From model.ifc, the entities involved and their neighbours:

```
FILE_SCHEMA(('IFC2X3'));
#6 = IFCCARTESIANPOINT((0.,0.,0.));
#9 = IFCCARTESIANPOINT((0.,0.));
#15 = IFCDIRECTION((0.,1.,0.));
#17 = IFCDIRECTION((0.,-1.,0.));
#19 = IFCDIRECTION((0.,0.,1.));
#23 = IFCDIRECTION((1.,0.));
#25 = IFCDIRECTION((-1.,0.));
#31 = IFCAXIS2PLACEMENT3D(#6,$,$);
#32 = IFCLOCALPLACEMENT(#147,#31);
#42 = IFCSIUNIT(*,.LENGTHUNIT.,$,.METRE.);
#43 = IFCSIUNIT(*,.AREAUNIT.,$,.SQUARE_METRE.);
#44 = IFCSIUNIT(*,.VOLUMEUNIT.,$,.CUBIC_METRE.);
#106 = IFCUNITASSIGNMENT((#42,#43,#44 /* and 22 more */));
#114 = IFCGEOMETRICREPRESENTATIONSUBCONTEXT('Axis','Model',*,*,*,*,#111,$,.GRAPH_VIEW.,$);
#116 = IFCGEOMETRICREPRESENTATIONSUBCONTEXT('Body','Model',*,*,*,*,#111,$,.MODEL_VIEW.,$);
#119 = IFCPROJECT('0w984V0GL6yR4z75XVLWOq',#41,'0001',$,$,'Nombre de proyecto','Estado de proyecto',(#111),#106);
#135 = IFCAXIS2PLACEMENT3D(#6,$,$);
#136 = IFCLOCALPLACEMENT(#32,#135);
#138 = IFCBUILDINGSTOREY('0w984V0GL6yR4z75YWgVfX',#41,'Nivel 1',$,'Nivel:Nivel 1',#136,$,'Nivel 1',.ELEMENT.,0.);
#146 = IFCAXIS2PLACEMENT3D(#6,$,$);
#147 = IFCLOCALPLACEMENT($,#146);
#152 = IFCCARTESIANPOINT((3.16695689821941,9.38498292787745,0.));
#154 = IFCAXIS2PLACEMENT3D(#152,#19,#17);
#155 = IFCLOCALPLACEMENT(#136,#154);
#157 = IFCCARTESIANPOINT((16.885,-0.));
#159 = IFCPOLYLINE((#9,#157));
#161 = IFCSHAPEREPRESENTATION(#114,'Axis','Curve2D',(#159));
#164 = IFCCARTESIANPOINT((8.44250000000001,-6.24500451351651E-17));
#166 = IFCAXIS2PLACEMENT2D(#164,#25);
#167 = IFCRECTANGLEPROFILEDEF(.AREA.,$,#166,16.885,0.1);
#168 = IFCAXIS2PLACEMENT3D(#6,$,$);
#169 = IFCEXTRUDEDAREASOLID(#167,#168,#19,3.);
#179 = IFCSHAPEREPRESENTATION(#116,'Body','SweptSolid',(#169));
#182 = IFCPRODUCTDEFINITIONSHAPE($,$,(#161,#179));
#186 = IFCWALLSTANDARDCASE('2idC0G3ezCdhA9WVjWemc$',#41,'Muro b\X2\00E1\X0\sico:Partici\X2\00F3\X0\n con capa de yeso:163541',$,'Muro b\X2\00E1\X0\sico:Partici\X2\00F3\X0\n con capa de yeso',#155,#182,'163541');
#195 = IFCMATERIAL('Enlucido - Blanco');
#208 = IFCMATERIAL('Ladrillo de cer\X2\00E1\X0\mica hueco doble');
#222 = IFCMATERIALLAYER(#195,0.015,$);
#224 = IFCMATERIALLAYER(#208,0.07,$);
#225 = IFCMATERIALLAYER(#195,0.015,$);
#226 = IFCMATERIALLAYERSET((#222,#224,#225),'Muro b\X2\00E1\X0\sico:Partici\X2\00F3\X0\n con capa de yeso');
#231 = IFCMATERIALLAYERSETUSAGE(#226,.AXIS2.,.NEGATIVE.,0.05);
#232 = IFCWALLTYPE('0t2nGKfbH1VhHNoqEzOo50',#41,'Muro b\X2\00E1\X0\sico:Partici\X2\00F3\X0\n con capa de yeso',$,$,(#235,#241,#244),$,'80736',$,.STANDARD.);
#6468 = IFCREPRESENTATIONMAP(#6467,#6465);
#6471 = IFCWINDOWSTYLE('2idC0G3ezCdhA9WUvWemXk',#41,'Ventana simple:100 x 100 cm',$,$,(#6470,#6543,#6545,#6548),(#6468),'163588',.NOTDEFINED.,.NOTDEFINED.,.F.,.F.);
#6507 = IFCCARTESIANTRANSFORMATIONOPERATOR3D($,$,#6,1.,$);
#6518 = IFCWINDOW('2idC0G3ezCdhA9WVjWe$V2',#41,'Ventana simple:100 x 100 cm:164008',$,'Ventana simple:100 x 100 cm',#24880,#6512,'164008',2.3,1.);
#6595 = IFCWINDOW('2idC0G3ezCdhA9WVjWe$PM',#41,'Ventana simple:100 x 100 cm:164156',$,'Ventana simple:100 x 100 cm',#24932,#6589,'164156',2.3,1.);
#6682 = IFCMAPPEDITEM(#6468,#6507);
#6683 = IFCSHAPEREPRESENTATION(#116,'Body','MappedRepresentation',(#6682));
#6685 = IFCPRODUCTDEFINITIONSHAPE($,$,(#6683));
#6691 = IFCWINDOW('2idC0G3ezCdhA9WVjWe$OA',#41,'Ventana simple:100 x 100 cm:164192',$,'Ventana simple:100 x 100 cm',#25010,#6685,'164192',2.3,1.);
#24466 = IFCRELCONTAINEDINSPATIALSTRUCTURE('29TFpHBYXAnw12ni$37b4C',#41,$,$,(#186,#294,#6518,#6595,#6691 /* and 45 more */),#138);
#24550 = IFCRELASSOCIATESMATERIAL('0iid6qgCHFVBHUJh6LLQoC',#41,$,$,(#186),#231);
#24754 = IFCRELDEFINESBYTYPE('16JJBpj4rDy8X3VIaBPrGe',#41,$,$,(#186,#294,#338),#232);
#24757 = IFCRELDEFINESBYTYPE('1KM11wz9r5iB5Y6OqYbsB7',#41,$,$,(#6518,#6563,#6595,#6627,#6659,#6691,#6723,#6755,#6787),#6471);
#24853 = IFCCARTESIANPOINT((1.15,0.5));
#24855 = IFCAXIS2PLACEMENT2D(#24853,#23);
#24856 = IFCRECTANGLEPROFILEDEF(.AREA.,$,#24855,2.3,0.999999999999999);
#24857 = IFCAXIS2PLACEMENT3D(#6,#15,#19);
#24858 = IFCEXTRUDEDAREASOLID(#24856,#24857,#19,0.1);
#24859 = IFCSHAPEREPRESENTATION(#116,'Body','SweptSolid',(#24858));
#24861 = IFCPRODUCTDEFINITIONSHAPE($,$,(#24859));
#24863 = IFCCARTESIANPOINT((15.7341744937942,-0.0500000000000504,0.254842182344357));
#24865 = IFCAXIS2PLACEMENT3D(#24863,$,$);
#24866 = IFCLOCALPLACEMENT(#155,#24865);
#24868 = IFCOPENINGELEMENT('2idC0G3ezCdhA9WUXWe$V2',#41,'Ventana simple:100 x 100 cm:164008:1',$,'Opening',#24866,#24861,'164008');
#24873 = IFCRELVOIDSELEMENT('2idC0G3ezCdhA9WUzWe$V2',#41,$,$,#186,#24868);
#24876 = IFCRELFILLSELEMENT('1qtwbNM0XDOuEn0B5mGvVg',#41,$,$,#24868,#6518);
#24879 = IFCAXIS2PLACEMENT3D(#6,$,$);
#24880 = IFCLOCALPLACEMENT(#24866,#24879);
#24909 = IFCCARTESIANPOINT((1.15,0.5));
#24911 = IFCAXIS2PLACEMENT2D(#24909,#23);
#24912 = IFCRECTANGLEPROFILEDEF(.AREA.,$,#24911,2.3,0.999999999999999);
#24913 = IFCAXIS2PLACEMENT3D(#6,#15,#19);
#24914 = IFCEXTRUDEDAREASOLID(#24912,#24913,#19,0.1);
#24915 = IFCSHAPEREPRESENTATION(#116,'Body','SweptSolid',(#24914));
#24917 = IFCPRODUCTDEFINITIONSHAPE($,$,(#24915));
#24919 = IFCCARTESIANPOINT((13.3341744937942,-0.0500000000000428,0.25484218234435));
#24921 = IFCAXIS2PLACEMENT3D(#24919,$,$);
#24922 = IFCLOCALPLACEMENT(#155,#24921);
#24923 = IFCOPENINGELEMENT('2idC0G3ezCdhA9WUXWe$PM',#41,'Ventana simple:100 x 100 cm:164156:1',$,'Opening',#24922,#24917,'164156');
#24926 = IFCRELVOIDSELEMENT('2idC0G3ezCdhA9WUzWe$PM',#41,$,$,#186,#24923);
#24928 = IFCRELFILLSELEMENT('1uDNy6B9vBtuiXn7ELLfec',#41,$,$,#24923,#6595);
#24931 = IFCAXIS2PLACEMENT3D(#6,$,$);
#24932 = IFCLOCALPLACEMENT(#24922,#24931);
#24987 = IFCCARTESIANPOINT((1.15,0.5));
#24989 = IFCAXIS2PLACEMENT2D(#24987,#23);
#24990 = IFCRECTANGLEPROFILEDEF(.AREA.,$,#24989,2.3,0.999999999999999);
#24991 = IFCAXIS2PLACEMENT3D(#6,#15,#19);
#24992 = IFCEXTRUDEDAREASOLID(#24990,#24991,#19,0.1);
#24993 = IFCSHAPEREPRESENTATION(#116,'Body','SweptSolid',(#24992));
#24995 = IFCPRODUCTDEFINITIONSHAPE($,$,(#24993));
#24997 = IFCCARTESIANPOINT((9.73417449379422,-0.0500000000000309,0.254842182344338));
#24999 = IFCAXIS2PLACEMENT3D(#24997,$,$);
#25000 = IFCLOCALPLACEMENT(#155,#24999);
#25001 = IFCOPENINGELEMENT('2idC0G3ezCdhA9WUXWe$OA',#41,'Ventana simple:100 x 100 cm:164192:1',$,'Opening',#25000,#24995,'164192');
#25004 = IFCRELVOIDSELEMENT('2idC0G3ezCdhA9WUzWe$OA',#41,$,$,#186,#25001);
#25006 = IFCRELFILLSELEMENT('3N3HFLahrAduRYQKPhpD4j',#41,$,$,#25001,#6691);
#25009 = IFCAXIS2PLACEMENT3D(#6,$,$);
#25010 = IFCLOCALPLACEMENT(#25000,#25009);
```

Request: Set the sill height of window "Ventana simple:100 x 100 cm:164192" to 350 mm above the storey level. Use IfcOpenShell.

```python
import numpy as np
import ifcopenshell
import ifcopenshell.api.geometry
import ifcopenshell.geom
import ifcopenshell.util.element
import ifcopenshell.util.placement
import ifcopenshell.util.shape
import ifcopenshell.util.unit

model = ifcopenshell.open("model.ifc")
unit_scale = ifcopenshell.util.unit.calculate_unit_scale(model)

window = model.by_guid("2idC0G3ezCdhA9WVjWe$OA")
opening = window.FillsVoids[0].RelatingOpeningElement
storey = ifcopenshell.util.element.get_container(window, ifc_class="IfcBuildingStorey")
level = ifcopenshell.util.placement.get_local_placement(storey.ObjectPlacement)[2, 3]

# The opening's origin need not be at the sill, so measure its lowest point.
shape = ifcopenshell.geom.create_shape(ifcopenshell.geom.settings(), opening)
bottom = ifcopenshell.util.shape.get_shape_bottom_elevation(shape, shape.geometry) / unit_scale
dz = level + 0.35 / unit_scale - bottom

shift = np.array([0.0, 0.0, dz])
# The window is placed relative to its opening, so it follows when the opening moves.
matrix = ifcopenshell.util.placement.get_local_placement(opening.ObjectPlacement)
matrix[:3, 3] += shift
ifcopenshell.api.geometry.edit_object_placement(
    model, product=opening, matrix=matrix, is_si=False, should_transform_children=True
)

print(f"moved by {dz * unit_scale:+.3f} m")

model.write("model_rev.ifc")
```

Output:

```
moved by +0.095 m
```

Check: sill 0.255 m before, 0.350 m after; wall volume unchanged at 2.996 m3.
